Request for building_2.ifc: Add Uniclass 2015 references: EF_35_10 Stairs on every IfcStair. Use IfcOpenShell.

First a look at what the model holds.

```python
import ifcopenshell

model = ifcopenshell.open("building_2.ifc")
print(model.schema)
print("classifications:", [c.Name for c in model.by_type("IfcClassification")])
for ifc_class in ("IfcDoor", "IfcRoof", "IfcStair", "IfcWall", "IfcWindow"):
    print(ifc_class, len(model.by_type(ifc_class)))
```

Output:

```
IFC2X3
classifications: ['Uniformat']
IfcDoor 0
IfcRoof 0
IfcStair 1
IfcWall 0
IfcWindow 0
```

```python
import ifcopenshell
import ifcopenshell.api.classification

model = ifcopenshell.open("building_2.ifc")

# IFC2X3 requires Source and Edition and has no link from the project to the system.
system = model.create_entity("IfcClassification", Source="NBS", Edition="2015", Name="Uniclass 2015")

codes = {
    "IfcStair": ("EF_35_10", "Stairs"),
}
for ifc_class, (code, name) in codes.items():
    products = model.by_type(ifc_class)
    ifcopenshell.api.classification.add_reference(
        model, products=products, classification=system, identification=code, name=name
    )
    print(code, len(products))

model.write("building_2_edited.ifc")
```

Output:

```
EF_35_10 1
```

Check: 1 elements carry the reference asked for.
